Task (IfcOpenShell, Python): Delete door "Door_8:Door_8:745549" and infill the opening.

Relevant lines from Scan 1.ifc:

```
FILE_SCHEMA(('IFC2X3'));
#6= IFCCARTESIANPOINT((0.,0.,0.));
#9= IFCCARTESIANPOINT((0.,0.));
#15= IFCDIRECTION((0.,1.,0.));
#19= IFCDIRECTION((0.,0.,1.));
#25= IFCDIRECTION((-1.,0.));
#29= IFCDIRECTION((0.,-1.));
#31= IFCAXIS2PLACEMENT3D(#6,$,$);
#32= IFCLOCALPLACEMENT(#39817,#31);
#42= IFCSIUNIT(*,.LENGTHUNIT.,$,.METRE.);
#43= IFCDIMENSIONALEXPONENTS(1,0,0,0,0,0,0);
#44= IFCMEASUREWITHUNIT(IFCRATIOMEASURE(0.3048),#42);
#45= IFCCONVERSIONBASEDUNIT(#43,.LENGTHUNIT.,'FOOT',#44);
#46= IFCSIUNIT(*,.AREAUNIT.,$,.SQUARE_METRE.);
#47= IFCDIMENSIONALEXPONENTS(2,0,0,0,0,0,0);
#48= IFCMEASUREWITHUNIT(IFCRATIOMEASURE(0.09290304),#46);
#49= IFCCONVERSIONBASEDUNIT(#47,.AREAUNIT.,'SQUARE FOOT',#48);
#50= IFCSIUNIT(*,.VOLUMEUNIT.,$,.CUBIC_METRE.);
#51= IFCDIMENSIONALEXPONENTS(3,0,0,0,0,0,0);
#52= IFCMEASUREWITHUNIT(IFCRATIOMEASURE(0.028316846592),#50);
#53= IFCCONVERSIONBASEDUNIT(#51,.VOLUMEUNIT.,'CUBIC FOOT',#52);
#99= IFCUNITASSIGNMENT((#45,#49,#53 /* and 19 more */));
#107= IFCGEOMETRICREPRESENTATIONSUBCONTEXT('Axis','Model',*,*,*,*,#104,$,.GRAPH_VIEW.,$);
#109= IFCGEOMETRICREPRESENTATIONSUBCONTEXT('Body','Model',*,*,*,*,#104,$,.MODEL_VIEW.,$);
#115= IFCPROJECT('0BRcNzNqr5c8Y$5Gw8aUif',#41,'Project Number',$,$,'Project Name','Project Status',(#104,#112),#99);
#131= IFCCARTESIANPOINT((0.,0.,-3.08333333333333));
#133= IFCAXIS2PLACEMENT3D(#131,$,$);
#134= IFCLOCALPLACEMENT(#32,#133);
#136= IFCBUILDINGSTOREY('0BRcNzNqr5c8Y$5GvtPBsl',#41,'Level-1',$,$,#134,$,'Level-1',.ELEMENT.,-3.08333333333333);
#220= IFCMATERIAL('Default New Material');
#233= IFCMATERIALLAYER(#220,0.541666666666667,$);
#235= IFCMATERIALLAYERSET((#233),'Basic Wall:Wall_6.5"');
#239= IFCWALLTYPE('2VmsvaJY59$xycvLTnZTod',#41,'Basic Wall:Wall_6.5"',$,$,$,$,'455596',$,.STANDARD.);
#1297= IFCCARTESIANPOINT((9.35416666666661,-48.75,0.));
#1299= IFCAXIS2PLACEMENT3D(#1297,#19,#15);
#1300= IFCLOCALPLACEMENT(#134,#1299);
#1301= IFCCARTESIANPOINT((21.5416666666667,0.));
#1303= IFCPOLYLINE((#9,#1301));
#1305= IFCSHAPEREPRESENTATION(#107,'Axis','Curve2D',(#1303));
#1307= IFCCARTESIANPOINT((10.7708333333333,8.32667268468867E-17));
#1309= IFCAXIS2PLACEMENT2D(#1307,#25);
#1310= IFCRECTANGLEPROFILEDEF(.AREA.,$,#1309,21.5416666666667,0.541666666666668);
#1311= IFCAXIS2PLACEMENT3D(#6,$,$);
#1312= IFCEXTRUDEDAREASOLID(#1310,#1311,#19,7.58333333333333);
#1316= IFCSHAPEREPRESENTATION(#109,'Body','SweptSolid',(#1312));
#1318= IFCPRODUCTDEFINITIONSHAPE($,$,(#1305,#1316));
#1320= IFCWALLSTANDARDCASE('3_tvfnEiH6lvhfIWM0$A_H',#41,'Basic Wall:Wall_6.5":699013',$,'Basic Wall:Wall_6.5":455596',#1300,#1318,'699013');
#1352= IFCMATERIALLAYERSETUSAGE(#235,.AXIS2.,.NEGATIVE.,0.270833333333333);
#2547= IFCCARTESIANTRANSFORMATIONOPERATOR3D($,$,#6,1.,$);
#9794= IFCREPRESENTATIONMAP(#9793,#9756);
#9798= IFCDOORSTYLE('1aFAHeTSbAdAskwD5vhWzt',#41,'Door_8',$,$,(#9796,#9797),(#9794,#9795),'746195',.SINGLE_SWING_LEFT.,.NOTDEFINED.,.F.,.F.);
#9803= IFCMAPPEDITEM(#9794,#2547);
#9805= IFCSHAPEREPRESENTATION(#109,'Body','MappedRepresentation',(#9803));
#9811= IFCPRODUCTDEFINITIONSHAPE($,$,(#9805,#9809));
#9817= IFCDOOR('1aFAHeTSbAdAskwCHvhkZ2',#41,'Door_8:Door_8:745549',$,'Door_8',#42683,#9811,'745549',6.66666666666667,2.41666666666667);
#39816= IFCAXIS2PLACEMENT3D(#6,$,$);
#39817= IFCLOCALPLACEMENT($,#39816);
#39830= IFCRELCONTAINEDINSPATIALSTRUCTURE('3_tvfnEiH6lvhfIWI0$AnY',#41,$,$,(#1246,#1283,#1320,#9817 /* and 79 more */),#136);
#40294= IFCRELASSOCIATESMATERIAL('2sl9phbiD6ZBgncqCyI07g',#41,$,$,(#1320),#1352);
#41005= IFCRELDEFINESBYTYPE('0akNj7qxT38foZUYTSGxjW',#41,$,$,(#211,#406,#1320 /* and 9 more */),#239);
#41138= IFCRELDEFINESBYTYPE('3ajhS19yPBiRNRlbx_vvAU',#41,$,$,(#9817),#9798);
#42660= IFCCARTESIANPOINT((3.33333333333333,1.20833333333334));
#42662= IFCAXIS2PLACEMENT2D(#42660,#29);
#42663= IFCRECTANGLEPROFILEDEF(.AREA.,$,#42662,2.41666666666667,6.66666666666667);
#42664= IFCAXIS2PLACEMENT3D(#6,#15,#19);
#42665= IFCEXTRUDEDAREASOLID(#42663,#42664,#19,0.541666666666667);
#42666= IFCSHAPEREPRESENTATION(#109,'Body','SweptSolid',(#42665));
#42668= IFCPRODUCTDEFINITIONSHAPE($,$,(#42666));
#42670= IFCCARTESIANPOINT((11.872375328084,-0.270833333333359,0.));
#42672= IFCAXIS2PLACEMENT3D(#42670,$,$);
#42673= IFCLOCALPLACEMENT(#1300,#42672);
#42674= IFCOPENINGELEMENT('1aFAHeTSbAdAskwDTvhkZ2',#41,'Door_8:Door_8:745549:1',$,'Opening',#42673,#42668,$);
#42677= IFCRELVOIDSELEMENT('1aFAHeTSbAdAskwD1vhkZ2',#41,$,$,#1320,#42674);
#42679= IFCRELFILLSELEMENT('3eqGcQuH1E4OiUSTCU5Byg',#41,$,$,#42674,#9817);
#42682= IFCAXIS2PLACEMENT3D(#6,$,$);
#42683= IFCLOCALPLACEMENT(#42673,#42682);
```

```python
import ifcopenshell
import ifcopenshell.api.feature
import ifcopenshell.api.root
import ifcopenshell.geom
import ifcopenshell.util.shape

model = ifcopenshell.open("Scan 1.ifc")
settings = ifcopenshell.geom.settings()


def volume(element):
    """Net volume in cubic metres, openings subtracted."""
    shape = ifcopenshell.geom.create_shape(settings, element)
    return ifcopenshell.util.shape.get_volume(shape.geometry)


door = model.by_guid("1aFAHeTSbAdAskwCHvhkZ2")
opening = door.FillsVoids[0].RelatingOpeningElement
wall = opening.VoidsElements[0].RelatingBuildingElement
before = volume(wall)

ifcopenshell.api.root.remove_product(model, product=door)
ifcopenshell.api.feature.remove_feature(model, feature=opening)

after = volume(wall)

print(f"wall volume {before:.3f} -> {after:.3f} m3")

model.write("Scan 1-out.ifc")
```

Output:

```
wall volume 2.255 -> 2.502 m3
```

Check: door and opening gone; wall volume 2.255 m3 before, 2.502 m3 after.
